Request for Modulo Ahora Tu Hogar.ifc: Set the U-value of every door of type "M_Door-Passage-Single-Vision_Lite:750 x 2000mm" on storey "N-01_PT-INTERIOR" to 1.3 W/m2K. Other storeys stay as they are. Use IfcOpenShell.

First a look at what the model holds.

```python
import ifcopenshell
import ifcopenshell.util.element

model = ifcopenshell.open("Modulo Ahora Tu Hogar.ifc")
print(model.schema)
storey = next(s for s in model.by_type("IfcBuildingStorey") if s.Name == "N-01_PT-INTERIOR")
doors = [e for e in ifcopenshell.util.element.get_decomposition(storey) if e.is_a("IfcDoor")]
seen = {}
for e in doors:
    element_type = ifcopenshell.util.element.get_type(e)
    key = (element_type.Name if element_type != e and element_type else None, ifcopenshell.util.element.get_pset(e, "Pset_DoorCommon", "ThermalTransmittance"))
    seen[key] = seen.get(key, 0) + 1
for (name, value), count in sorted(seen.items(), key=str):
    print(count, "x", name, "|", value)
```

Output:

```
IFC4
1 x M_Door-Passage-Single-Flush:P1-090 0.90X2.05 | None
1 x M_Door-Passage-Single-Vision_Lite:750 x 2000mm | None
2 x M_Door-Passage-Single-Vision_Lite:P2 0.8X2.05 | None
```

```python
import ifcopenshell
import ifcopenshell.api.pset
import ifcopenshell.util.element

model = ifcopenshell.open("Modulo Ahora Tu Hogar.ifc")

storey = next(s for s in model.by_type("IfcBuildingStorey") if s.Name == "N-01_PT-INTERIOR")
doors = [e for e in ifcopenshell.util.element.get_decomposition(storey) if e.is_a("IfcDoor")]

count = 0
for e in doors:
    element_type = ifcopenshell.util.element.get_type(e)
    if element_type in (None, e) or element_type.Name != "M_Door-Passage-Single-Vision_Lite:750 x 2000mm":
        continue
    # add_pset returns the element's existing set when there is one.
    pset = ifcopenshell.api.pset.add_pset(model, product=e, name="Pset_DoorCommon")
    ifcopenshell.api.pset.edit_pset(model, pset=pset, properties={"ThermalTransmittance": 1.3})
    count += 1

print(count, "doors updated")

model.write("Modulo Ahora Tu Hogar_updated.ifc")
```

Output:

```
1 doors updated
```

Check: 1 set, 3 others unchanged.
